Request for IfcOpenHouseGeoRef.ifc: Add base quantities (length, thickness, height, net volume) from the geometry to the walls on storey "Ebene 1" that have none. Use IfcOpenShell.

First a look at what the model holds.

```python
import ifcopenshell
import ifcopenshell.util.element
import ifcopenshell.util.unit

model = ifcopenshell.open("IfcOpenHouseGeoRef.ifc")
print(model.schema)
for unit_type in ("LENGTHUNIT", "AREAUNIT", "VOLUMEUNIT"):
    print(unit_type, ifcopenshell.util.unit.calculate_unit_scale(model, unit_type))
storey = next(s for s in model.by_type("IfcBuildingStorey") if s.Name == "Ebene 1")
walls = [e for e in ifcopenshell.util.element.get_decomposition(storey) if e.is_a("IfcWall")]
for e in sorted(walls, key=lambda e: e.id()):
    print(e.id(), e.is_a(), e.Name, list(ifcopenshell.util.element.get_psets(e, qtos_only=True)), sep=" | ")
```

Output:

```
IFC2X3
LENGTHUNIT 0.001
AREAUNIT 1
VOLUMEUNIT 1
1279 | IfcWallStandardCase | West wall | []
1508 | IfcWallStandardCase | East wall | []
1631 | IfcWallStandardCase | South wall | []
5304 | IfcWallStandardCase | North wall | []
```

```python
import ifcopenshell
import ifcopenshell.api.pset
import ifcopenshell.geom
import ifcopenshell.util.element
import ifcopenshell.util.shape
import ifcopenshell.util.unit

model = ifcopenshell.open("IfcOpenHouseGeoRef.ifc")
unit_scale = ifcopenshell.util.unit.calculate_unit_scale(model)
volume_scale = ifcopenshell.util.unit.calculate_unit_scale(model, "VOLUMEUNIT")
settings = ifcopenshell.geom.settings()

storey = next(s for s in model.by_type("IfcBuildingStorey") if s.Name == "Ebene 1")
walls = [e for e in ifcopenshell.util.element.get_decomposition(storey) if e.is_a("IfcWall")]

for e in sorted(walls, key=lambda e: e.id()):
    if ifcopenshell.util.element.get_psets(e, qtos_only=True, should_inherit=False):
        continue
    # Geometry comes back in metres, in the element's own axes.
    shape = ifcopenshell.geom.create_shape(settings, e)
    values = {
        "Length": ifcopenshell.util.shape.get_x(shape.geometry) / unit_scale,
        "Width": ifcopenshell.util.shape.get_y(shape.geometry) / unit_scale,
        "Height": ifcopenshell.util.shape.get_z(shape.geometry) / unit_scale,
        "NetVolume": ifcopenshell.util.shape.get_volume(shape.geometry) / volume_scale,
    }
    qto = ifcopenshell.api.pset.add_qto(model, product=e, name="BaseQuantities")
    ifcopenshell.api.pset.edit_qto(model, qto=qto, properties=values)
    print(e.id(), {k: round(v, 3) for k, v in values.items()})

model.write("IfcOpenHouseGeoRef_updated.ifc")
```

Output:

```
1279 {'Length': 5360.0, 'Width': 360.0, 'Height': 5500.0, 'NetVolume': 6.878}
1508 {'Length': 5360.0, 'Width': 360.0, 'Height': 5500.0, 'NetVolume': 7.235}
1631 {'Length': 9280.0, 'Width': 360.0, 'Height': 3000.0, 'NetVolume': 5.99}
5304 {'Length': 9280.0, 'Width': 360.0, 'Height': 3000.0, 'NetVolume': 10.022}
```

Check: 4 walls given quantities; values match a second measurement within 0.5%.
